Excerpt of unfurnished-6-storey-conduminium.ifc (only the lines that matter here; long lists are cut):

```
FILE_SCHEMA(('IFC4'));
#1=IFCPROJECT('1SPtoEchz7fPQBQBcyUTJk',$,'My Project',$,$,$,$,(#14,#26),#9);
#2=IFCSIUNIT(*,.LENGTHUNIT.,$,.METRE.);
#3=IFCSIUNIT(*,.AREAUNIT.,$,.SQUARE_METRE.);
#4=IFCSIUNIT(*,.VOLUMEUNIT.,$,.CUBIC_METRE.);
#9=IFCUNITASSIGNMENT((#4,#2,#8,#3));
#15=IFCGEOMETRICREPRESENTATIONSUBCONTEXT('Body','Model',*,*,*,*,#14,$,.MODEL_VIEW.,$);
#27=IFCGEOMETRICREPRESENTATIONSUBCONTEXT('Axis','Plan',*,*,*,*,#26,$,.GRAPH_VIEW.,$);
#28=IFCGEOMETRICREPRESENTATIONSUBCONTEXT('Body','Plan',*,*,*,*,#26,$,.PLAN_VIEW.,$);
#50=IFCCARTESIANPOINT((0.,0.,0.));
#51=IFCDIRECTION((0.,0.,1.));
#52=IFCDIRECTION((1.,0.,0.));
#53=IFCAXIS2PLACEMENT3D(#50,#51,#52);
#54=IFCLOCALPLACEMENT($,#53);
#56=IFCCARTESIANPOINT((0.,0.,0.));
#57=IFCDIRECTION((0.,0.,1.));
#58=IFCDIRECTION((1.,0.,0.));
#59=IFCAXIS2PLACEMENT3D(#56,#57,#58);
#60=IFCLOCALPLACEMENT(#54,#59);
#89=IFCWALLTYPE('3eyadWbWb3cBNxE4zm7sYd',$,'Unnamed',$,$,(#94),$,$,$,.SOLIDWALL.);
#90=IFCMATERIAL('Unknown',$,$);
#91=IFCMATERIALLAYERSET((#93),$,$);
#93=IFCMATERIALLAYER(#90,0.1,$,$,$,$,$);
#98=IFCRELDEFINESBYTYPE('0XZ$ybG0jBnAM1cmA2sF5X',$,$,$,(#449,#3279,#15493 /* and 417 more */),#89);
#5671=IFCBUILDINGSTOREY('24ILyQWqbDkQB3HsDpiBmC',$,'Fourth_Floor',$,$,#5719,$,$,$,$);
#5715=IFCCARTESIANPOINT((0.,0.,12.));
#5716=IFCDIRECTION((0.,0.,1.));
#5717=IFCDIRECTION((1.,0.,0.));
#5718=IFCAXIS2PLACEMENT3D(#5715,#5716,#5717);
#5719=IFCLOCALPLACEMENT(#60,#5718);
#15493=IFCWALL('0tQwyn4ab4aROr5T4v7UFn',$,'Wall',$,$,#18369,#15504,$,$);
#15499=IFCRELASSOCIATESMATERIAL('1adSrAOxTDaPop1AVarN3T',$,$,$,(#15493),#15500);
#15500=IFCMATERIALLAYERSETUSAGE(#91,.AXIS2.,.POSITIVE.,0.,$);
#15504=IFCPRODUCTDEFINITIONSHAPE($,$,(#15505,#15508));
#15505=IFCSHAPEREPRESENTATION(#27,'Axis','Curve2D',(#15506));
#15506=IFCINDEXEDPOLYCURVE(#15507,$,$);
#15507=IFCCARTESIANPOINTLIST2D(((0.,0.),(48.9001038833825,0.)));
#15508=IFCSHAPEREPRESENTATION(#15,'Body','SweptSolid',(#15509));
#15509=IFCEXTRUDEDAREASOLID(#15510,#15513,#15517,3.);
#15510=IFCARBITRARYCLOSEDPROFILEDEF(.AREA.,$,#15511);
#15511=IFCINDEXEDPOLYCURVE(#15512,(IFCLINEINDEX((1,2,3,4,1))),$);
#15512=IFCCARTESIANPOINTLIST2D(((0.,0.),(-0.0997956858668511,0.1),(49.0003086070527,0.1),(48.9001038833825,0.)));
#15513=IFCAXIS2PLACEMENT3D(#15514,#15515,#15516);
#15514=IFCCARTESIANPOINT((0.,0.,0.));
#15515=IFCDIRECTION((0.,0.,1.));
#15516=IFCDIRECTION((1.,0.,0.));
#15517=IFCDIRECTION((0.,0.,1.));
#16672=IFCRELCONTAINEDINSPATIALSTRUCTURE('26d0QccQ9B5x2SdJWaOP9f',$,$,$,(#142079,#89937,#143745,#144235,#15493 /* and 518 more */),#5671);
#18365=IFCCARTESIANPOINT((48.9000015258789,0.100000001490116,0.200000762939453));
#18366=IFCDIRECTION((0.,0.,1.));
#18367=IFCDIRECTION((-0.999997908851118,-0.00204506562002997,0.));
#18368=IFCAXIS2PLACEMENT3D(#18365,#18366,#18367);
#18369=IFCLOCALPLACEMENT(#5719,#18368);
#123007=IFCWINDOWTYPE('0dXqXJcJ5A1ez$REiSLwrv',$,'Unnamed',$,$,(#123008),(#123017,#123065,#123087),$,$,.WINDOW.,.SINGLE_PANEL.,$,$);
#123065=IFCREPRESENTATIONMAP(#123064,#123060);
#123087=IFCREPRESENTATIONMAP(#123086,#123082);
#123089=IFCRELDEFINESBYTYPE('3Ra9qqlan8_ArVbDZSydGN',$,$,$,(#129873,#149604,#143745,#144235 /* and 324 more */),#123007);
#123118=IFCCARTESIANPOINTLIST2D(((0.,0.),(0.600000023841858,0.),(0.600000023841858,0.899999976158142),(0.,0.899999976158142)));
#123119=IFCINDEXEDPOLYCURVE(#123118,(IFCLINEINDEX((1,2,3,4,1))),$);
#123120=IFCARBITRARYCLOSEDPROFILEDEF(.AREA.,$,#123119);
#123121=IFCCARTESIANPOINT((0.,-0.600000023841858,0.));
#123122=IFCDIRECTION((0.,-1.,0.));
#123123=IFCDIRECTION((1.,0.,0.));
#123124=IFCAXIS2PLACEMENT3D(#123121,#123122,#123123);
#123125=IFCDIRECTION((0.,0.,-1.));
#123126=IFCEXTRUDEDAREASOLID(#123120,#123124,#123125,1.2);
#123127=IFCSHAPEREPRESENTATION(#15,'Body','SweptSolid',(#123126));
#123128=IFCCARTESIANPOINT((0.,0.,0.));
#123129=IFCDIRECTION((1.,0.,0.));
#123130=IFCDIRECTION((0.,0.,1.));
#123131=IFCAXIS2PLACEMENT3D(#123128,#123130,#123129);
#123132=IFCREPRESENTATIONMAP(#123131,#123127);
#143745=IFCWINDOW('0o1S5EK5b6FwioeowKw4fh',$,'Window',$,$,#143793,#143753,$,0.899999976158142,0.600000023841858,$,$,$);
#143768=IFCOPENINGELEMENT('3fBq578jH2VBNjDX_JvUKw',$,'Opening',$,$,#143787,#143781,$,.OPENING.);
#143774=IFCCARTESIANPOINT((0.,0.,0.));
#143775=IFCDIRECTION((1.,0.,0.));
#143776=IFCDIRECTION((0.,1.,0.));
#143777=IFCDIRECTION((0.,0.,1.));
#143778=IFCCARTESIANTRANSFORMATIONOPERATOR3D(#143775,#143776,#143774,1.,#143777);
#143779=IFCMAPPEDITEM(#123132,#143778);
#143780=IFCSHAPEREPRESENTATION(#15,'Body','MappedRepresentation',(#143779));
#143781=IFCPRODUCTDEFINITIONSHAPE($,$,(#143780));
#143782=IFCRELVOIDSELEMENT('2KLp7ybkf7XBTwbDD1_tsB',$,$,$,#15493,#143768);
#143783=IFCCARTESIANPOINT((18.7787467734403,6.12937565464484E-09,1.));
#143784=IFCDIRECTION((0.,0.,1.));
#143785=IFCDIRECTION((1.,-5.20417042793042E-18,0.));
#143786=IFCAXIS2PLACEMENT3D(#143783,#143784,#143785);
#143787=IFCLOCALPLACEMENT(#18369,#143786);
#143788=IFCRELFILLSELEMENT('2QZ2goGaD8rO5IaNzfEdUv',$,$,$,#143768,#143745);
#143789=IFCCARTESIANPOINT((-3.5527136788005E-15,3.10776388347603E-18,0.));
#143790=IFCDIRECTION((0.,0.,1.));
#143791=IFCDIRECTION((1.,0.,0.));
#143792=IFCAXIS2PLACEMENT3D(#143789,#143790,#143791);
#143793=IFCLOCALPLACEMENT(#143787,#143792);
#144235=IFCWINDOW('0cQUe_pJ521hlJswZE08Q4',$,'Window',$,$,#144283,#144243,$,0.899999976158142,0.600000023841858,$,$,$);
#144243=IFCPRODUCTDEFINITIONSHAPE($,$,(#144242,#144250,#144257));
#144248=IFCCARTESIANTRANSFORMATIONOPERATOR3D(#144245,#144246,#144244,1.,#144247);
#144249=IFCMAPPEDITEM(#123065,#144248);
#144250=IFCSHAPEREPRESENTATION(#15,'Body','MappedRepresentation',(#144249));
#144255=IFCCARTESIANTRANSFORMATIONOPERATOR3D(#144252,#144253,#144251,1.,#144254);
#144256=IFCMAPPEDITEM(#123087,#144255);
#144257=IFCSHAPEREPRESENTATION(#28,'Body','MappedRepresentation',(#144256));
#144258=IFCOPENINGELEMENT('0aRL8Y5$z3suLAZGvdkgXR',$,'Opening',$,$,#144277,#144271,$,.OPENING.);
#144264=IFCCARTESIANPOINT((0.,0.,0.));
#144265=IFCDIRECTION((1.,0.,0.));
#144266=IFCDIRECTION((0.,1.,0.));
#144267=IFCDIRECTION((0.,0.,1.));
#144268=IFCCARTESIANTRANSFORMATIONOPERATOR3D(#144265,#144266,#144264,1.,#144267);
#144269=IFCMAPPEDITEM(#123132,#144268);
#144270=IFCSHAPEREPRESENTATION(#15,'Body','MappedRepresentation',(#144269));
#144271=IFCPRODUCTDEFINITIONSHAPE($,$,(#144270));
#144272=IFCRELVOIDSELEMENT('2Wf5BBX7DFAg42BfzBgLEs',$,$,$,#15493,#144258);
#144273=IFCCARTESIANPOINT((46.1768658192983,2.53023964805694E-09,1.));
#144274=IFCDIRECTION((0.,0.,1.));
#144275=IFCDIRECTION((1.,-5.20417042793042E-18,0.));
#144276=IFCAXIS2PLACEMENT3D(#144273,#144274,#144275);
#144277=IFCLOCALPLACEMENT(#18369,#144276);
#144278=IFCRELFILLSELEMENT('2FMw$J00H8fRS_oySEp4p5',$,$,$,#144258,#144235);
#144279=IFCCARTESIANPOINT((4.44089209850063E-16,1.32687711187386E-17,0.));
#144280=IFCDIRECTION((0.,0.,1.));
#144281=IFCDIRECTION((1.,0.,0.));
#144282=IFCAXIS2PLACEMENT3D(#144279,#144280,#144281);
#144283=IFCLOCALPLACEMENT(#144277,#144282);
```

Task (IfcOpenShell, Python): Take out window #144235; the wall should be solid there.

```python
import ifcopenshell
import ifcopenshell.api.feature
import ifcopenshell.api.root
import ifcopenshell.geom
import ifcopenshell.util.shape

model = ifcopenshell.open("unfurnished-6-storey-conduminium.ifc")
settings = ifcopenshell.geom.settings()


def volume(element):
    """Net volume in cubic metres, openings subtracted."""
    shape = ifcopenshell.geom.create_shape(settings, element)
    return ifcopenshell.util.shape.get_volume(shape.geometry)


window = model.by_id(144235)
opening = window.FillsVoids[0].RelatingOpeningElement
wall = opening.VoidsElements[0].RelatingBuildingElement
before = volume(wall)

ifcopenshell.api.root.remove_product(model, product=window)
ifcopenshell.api.feature.remove_feature(model, feature=opening)

after = volume(wall)

print(f"wall volume {before:.3f} -> {after:.3f} m3")

model.write("unfurnished-6-storey-conduminium_updated.ifc")
```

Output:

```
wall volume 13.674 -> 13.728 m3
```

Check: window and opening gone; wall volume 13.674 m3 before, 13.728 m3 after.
